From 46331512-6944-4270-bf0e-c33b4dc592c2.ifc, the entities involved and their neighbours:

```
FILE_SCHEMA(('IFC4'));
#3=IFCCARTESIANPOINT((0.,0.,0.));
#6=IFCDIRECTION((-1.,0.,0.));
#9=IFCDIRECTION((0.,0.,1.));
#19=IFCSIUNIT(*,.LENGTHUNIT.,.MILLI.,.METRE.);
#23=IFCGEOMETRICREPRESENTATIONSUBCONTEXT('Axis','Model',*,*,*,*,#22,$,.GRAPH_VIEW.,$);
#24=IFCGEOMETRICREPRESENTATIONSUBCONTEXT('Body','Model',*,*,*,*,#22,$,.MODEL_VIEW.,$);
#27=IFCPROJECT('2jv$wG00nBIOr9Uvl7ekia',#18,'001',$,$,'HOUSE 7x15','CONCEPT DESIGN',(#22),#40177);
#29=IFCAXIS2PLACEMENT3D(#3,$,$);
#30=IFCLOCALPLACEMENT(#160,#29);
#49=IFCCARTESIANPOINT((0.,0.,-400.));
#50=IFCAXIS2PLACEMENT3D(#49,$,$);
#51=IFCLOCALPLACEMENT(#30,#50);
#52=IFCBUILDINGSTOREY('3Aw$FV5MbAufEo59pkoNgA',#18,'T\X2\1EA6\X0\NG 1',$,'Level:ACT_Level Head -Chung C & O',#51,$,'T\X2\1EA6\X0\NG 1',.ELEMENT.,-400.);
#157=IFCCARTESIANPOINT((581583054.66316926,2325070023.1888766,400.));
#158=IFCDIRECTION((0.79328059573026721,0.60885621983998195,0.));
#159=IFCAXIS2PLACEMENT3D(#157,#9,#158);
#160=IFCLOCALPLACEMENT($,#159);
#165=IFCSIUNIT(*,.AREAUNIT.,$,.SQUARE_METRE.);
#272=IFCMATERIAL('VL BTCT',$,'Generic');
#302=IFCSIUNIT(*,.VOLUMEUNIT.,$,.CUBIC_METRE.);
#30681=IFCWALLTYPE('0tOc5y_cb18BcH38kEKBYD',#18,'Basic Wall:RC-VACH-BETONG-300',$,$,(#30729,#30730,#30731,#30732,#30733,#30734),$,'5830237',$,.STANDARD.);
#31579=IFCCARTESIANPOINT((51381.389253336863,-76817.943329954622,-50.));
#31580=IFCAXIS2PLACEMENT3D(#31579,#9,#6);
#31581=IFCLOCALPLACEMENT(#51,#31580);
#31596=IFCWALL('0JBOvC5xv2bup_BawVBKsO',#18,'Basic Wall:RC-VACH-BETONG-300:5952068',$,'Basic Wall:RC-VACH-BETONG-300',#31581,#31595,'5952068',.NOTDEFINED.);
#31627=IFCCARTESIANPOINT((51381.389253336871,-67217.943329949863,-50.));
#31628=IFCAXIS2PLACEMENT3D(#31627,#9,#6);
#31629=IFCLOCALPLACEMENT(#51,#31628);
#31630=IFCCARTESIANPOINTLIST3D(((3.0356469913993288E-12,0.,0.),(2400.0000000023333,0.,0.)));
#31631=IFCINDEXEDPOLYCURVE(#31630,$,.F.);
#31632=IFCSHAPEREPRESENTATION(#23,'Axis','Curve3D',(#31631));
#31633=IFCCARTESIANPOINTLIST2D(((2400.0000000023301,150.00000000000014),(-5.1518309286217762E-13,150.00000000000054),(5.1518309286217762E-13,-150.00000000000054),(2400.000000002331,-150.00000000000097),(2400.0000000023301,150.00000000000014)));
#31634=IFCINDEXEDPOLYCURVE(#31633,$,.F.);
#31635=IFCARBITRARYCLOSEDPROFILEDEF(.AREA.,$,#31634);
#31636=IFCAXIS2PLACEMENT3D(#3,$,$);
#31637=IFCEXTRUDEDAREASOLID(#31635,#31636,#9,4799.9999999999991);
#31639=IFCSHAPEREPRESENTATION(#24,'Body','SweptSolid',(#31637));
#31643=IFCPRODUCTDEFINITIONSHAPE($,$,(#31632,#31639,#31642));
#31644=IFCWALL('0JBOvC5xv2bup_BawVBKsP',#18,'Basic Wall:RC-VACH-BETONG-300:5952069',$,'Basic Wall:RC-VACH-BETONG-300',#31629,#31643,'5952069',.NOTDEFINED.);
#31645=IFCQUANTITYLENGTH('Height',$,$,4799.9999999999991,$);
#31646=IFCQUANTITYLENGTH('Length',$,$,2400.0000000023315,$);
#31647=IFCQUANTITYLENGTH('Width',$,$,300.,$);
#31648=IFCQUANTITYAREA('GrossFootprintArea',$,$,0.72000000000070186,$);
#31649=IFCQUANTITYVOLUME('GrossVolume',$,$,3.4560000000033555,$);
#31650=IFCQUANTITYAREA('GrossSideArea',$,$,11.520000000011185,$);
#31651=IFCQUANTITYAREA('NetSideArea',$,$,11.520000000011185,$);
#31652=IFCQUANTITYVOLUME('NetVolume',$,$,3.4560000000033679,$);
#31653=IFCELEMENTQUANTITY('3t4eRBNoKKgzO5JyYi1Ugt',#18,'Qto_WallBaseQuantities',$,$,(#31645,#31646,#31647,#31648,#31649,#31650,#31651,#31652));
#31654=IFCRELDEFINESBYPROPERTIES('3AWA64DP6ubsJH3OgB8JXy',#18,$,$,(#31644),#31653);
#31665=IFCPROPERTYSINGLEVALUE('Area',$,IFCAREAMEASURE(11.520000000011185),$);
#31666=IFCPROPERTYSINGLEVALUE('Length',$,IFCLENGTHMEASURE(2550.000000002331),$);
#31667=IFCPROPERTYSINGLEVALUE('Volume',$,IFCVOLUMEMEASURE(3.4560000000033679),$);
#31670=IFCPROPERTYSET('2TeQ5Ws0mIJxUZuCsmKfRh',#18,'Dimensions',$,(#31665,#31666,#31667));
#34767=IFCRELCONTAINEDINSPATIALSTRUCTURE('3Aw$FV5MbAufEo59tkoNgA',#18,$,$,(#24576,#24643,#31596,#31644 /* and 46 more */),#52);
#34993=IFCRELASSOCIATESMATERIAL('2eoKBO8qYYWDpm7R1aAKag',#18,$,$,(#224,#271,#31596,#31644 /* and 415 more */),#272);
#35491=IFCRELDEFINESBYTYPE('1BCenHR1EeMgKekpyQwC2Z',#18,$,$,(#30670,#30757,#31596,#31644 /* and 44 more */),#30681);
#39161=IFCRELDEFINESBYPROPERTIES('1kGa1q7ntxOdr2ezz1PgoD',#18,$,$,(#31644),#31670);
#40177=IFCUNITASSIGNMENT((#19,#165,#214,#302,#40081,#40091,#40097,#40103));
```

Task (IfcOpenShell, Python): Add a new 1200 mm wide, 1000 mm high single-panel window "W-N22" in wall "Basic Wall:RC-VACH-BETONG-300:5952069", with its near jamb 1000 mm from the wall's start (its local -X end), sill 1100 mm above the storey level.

```python
import numpy as np
import ifcopenshell
import ifcopenshell.api.feature
import ifcopenshell.api.geometry
import ifcopenshell.api.pset
import ifcopenshell.api.root
import ifcopenshell.api.spatial
import ifcopenshell.geom
import ifcopenshell.util.element
import ifcopenshell.util.placement
import ifcopenshell.util.representation
import ifcopenshell.util.shape
import ifcopenshell.util.unit

model = ifcopenshell.open("46331512-6944-4270-bf0e-c33b4dc592c2.ifc")
unit_scale = ifcopenshell.util.unit.calculate_unit_scale(model)
area_scale = ifcopenshell.util.unit.calculate_unit_scale(model, "AREAUNIT")
volume_scale = ifcopenshell.util.unit.calculate_unit_scale(model, "VOLUMEUNIT")
settings = ifcopenshell.geom.settings()


def volume(element):
    """Net volume in cubic metres, openings subtracted."""
    shape = ifcopenshell.geom.create_shape(settings, element)
    return ifcopenshell.util.shape.get_volume(shape.geometry)


wall = model.by_guid("0JBOvC5xv2bup_BawVBKsP")
storey = ifcopenshell.util.element.get_container(wall, ifc_class="IfcBuildingStorey")
context = ifcopenshell.util.representation.get_context(model, "Model", "Body", "MODEL_VIEW")
before = volume(wall)

width, height, from_end, sill = 1.2, 1, 1, 1.1  # metres

# The wall runs along its own X axis, and the end named is its -X end.
wall_shape = ifcopenshell.geom.create_shape(settings, wall)
x, y, z = ifcopenshell.util.shape.get_vertices(wall_shape.geometry).T
start = x.min() + from_end
face, thickness = float(y.min()), float(y.max() - y.min())
wall_matrix = ifcopenshell.util.placement.get_local_placement(wall.ObjectPlacement)
level = ifcopenshell.util.placement.get_local_placement(storey.ObjectPlacement)[2, 3]


def in_wall(x, y):
    """Placement at x, y metres in the wall's axes, at sill height."""
    matrix = wall_matrix.copy()
    matrix[:, 3] = wall_matrix @ np.array([x / unit_scale, y / unit_scale, 0.0, 1.0])
    matrix[2, 3] = level + sill / unit_scale
    return matrix


# Opening: a box that overshoots both wall faces by 50 mm.
opening = ifcopenshell.api.root.create_entity(model, ifc_class="IfcOpeningElement", predefined_type="OPENING")
box = ifcopenshell.api.geometry.add_wall_representation(
    model, context=context, length=width, height=height, thickness=thickness + 0.1
)
ifcopenshell.api.geometry.assign_representation(model, product=opening, representation=box)
ifcopenshell.api.geometry.edit_object_placement(model, product=opening, matrix=in_wall(start, face - 0.05), is_si=False)
ifcopenshell.api.feature.add_feature(model, feature=opening, element=wall)

window = ifcopenshell.api.root.create_entity(model, ifc_class="IfcWindow", name="W-N22", predefined_type="WINDOW")
window.OverallWidth, window.OverallHeight = width / unit_scale, height / unit_scale
window.PartitioningType = "SINGLE_PANEL"
body = ifcopenshell.api.geometry.add_window_representation(
    model,
    context=context,
    overall_width=window.OverallWidth,
    overall_height=window.OverallHeight,
    partition_type="SINGLE_PANEL",
)
ifcopenshell.api.geometry.assign_representation(model, product=window, representation=body)
ifcopenshell.api.spatial.assign_container(model, products=[window], relating_structure=storey)
ifcopenshell.api.feature.add_filling(model, opening=opening, element=window)

# Centre the window in the wall's thickness.
ifcopenshell.api.geometry.edit_object_placement(model, product=window, matrix=in_wall(start, face), is_si=False)
window_shape = ifcopenshell.geom.create_shape(settings, window)
depth = ifcopenshell.util.shape.get_vertices(window_shape.geometry)[:, 1]
offset = face + thickness / 2 - (depth.min() + depth.max()) / 2
ifcopenshell.api.geometry.edit_object_placement(model, product=window, matrix=in_wall(start, offset), is_si=False)

after = volume(wall)

# Update the wall's stored quantities.
qto = model.by_id(ifcopenshell.util.element.get_pset(wall, "Qto_WallBaseQuantities", should_inherit=False)["id"])
ifcopenshell.api.pset.edit_qto(model, qto=qto, properties={
    "NetSideArea": after / thickness / area_scale,
    "NetVolume": after / volume_scale,
})
pset = model.by_id(ifcopenshell.util.element.get_pset(wall, "Dimensions", should_inherit=False)["id"])
ifcopenshell.api.pset.edit_pset(model, pset=pset, properties={
    "Area": model.create_entity("IfcAreaMeasure", after / thickness / area_scale),
    "Volume": model.create_entity("IfcVolumeMeasure", after / volume_scale),
})

print(f"wall volume {before:.3f} -> {after:.3f} m3")

model.write("46331512-6944-4270-bf0e-c33b4dc592c2_rev.ifc")
```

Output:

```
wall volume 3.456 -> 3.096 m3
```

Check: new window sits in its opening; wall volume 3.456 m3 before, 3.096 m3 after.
